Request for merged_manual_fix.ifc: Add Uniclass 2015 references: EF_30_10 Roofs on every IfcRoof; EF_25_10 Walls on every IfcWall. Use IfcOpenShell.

First a look at what the model holds.

```python
import ifcopenshell

model = ifcopenshell.open("merged_manual_fix.ifc")
print(model.schema)
print("classifications:", [c.Name for c in model.by_type("IfcClassification")])
for ifc_class in ("IfcDoor", "IfcRoof", "IfcStair", "IfcWall", "IfcWindow"):
    print(ifc_class, len(model.by_type(ifc_class)))
```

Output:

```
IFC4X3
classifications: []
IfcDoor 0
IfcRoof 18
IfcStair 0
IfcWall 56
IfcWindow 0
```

```python
import ifcopenshell
import ifcopenshell.api.classification

model = ifcopenshell.open("merged_manual_fix.ifc")

system = ifcopenshell.api.classification.add_classification(model, classification="Uniclass 2015")

codes = {
    "IfcRoof": ("EF_30_10", "Roofs"),
    "IfcWall": ("EF_25_10", "Walls"),
}
for ifc_class, (code, name) in codes.items():
    products = model.by_type(ifc_class)
    ifcopenshell.api.classification.add_reference(
        model, products=products, classification=system, identification=code, name=name
    )
    print(code, len(products))

model.write("merged_manual_fix_updated.ifc")
```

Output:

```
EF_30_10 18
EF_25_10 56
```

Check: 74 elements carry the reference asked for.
